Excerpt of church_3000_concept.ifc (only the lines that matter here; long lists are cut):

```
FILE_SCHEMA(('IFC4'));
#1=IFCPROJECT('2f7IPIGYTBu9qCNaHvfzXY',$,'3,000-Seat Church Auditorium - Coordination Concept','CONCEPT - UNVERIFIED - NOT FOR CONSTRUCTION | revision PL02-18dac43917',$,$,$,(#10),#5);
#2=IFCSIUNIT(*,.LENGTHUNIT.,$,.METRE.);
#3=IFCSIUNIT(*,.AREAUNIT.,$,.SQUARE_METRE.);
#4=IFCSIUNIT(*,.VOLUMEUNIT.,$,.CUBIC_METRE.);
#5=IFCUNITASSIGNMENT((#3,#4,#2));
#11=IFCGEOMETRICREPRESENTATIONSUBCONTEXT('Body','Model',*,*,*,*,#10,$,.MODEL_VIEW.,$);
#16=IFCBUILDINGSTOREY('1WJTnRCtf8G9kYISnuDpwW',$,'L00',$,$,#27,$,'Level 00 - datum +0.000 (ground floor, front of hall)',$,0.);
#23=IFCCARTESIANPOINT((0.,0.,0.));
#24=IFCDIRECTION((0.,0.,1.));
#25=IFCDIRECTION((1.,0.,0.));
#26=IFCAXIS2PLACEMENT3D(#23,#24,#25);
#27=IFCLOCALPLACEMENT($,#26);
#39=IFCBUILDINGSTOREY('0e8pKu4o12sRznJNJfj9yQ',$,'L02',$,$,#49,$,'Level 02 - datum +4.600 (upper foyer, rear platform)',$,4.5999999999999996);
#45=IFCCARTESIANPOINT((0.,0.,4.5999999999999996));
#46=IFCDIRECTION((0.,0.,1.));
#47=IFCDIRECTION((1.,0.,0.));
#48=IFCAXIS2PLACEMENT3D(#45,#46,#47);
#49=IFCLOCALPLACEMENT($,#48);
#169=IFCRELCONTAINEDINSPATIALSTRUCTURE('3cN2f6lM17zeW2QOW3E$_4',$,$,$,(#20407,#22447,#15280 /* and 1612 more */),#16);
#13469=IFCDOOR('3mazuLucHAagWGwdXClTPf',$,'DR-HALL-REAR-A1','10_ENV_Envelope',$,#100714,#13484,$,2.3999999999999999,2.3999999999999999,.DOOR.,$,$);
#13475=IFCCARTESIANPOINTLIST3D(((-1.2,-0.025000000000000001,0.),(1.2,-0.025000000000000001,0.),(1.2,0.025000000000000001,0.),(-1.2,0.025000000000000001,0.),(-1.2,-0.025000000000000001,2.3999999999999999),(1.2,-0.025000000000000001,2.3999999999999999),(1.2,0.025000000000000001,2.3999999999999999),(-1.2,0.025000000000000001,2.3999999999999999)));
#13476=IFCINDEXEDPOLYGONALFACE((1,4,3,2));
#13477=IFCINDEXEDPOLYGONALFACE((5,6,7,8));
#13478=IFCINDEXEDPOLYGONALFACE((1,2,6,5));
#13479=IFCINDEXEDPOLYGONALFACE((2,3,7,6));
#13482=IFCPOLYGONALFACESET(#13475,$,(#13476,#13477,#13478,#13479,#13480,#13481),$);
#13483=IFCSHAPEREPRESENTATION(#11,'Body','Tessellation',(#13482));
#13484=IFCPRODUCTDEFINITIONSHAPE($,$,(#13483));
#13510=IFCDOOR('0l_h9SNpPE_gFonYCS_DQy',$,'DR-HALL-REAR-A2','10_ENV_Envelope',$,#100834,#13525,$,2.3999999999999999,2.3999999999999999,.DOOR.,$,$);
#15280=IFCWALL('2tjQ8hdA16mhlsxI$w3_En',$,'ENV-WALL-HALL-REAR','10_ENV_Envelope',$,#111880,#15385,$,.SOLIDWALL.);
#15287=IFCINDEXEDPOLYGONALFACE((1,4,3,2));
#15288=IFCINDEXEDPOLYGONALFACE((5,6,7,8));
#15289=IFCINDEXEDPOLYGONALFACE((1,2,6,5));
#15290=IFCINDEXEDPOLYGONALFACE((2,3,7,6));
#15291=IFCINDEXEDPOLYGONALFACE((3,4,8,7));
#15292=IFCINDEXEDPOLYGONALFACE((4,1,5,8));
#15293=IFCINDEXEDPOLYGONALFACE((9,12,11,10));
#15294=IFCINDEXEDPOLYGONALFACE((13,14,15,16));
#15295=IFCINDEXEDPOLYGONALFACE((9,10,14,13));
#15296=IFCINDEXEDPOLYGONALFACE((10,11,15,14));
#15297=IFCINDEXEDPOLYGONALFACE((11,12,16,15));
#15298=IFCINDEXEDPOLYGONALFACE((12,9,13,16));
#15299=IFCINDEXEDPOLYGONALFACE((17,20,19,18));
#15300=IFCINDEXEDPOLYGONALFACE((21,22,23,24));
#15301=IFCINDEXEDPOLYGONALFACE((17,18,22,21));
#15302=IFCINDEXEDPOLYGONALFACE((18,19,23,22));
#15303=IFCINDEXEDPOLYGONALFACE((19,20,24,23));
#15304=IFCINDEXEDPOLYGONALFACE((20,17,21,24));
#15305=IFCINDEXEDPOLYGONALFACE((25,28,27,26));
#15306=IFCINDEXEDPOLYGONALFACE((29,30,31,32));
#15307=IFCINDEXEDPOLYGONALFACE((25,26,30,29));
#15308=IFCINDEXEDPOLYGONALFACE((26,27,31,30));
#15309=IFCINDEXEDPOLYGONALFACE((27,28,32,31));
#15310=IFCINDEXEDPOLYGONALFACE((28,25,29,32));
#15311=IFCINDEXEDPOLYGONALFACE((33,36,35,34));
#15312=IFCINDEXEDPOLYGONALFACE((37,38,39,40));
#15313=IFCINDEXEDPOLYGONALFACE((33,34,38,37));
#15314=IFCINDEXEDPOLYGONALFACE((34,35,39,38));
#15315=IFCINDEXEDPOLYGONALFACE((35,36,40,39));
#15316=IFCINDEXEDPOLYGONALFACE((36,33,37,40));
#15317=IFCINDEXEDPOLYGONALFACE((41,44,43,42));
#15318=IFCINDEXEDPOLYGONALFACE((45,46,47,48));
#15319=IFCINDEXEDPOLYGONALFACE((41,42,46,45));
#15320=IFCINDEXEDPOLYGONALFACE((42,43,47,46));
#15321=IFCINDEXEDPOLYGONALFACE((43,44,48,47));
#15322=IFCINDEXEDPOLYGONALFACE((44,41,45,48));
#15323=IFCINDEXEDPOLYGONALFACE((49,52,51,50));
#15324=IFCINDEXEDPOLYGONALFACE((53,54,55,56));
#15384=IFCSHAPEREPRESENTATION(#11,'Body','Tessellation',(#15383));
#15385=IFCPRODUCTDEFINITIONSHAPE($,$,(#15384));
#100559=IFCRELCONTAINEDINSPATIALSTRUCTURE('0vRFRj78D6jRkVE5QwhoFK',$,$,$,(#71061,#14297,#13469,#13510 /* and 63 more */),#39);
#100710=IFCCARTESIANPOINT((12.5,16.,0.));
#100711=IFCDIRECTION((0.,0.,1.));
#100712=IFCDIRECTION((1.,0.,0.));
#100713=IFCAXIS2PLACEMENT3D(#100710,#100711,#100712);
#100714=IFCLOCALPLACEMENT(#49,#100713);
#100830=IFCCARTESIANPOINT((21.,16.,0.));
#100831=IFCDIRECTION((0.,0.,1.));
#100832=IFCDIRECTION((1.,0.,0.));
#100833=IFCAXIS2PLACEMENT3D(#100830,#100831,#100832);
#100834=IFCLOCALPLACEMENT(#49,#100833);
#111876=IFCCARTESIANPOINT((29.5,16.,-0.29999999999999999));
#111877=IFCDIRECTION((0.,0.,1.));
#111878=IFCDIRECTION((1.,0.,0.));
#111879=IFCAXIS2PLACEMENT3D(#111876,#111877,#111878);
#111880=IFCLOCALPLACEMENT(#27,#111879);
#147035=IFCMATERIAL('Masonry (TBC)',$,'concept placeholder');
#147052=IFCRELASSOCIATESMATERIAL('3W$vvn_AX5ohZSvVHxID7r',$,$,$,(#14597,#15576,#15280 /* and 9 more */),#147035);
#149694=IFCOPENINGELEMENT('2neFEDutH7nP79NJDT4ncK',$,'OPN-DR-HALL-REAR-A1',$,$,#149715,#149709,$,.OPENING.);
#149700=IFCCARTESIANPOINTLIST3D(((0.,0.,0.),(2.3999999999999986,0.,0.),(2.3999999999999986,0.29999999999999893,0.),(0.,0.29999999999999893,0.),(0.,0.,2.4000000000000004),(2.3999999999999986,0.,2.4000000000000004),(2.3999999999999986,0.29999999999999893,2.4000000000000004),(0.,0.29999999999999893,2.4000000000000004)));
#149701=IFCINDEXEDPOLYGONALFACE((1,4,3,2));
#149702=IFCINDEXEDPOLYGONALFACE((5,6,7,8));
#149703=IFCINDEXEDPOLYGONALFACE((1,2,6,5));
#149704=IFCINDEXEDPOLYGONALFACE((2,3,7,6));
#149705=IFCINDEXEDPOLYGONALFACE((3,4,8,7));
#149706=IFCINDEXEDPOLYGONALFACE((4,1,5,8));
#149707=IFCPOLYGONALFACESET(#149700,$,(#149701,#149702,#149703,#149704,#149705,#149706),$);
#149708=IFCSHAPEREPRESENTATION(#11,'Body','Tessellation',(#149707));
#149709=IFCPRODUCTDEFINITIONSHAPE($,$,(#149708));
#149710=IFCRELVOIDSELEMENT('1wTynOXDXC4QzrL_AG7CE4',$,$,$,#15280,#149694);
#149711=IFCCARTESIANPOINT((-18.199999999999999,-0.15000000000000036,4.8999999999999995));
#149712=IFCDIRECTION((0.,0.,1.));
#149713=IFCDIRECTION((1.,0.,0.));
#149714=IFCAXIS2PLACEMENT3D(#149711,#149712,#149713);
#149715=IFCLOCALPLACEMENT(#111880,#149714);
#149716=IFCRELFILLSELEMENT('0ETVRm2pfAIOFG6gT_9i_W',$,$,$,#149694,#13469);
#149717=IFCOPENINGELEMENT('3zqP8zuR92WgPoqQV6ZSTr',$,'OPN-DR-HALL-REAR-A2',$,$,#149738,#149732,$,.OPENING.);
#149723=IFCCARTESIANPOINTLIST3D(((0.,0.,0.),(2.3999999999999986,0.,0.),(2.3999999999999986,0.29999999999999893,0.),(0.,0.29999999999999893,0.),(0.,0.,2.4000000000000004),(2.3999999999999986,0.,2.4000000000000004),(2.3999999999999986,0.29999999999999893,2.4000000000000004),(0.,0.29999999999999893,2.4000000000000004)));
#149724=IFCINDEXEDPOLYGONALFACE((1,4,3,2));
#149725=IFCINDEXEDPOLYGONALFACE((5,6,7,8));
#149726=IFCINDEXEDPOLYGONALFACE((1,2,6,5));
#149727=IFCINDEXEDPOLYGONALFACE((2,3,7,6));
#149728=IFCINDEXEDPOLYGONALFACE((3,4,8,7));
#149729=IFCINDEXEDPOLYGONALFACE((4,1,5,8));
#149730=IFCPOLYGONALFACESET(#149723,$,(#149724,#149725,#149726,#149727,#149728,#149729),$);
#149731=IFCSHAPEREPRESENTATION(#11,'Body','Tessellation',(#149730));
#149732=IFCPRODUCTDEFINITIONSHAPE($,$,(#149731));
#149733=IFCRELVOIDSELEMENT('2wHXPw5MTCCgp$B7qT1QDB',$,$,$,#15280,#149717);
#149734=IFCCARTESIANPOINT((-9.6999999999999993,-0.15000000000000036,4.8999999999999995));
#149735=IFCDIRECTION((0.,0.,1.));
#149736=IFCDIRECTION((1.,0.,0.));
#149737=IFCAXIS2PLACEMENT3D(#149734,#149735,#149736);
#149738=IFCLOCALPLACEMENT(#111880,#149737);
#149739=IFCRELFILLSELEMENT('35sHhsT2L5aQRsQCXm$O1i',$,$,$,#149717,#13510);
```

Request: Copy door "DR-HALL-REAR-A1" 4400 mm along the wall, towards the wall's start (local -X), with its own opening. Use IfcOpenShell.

```python
import ifcopenshell
import ifcopenshell.api.feature
import ifcopenshell.api.geometry
import ifcopenshell.api.root
import ifcopenshell.geom
import ifcopenshell.util.element
import ifcopenshell.util.placement
import ifcopenshell.util.shape
import ifcopenshell.util.unit

model = ifcopenshell.open("church_3000_concept.ifc")
unit_scale = ifcopenshell.util.unit.calculate_unit_scale(model)
settings = ifcopenshell.geom.settings()


def volume(element):
    """Net volume in cubic metres, openings subtracted."""
    shape = ifcopenshell.geom.create_shape(settings, element)
    return ifcopenshell.util.shape.get_volume(shape.geometry)


door = model.by_guid("3mazuLucHAagWGwdXClTPf")
opening = door.FillsVoids[0].RelatingOpeningElement
wall = opening.VoidsElements[0].RelatingBuildingElement
before = volume(wall)
shift = ifcopenshell.util.placement.get_local_placement(wall.ObjectPlacement)[:3, 0] * -4.4 / unit_scale

# copy_class copies the void relationship, type, container and properties, but no geometry.
new_opening = ifcopenshell.api.root.copy_class(model, product=opening)
new_opening.Representation = ifcopenshell.util.element.copy_deep(
    model, opening.Representation, exclude=["IfcGeometricRepresentationContext", "IfcRepresentationMap"]
)
new_door = ifcopenshell.api.root.copy_class(model, product=door)
new_door.Representation = ifcopenshell.util.element.copy_deep(
    model, door.Representation, exclude=["IfcGeometricRepresentationContext", "IfcRepresentationMap"]
)
ifcopenshell.api.feature.add_filling(model, opening=new_opening, element=new_door)

for old, new in ((opening, new_opening), (door, new_door)):
    matrix = ifcopenshell.util.placement.get_local_placement(old.ObjectPlacement)
    matrix[:3, 3] += shift
    ifcopenshell.api.geometry.edit_object_placement(model, product=new, matrix=matrix, is_si=False)

after = volume(wall)

print(f"wall volume {before:.3f} -> {after:.3f} m3")

model.write("church_3000_concept_edited.ifc")
```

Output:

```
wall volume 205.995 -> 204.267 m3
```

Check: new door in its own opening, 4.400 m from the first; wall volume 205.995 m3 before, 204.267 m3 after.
